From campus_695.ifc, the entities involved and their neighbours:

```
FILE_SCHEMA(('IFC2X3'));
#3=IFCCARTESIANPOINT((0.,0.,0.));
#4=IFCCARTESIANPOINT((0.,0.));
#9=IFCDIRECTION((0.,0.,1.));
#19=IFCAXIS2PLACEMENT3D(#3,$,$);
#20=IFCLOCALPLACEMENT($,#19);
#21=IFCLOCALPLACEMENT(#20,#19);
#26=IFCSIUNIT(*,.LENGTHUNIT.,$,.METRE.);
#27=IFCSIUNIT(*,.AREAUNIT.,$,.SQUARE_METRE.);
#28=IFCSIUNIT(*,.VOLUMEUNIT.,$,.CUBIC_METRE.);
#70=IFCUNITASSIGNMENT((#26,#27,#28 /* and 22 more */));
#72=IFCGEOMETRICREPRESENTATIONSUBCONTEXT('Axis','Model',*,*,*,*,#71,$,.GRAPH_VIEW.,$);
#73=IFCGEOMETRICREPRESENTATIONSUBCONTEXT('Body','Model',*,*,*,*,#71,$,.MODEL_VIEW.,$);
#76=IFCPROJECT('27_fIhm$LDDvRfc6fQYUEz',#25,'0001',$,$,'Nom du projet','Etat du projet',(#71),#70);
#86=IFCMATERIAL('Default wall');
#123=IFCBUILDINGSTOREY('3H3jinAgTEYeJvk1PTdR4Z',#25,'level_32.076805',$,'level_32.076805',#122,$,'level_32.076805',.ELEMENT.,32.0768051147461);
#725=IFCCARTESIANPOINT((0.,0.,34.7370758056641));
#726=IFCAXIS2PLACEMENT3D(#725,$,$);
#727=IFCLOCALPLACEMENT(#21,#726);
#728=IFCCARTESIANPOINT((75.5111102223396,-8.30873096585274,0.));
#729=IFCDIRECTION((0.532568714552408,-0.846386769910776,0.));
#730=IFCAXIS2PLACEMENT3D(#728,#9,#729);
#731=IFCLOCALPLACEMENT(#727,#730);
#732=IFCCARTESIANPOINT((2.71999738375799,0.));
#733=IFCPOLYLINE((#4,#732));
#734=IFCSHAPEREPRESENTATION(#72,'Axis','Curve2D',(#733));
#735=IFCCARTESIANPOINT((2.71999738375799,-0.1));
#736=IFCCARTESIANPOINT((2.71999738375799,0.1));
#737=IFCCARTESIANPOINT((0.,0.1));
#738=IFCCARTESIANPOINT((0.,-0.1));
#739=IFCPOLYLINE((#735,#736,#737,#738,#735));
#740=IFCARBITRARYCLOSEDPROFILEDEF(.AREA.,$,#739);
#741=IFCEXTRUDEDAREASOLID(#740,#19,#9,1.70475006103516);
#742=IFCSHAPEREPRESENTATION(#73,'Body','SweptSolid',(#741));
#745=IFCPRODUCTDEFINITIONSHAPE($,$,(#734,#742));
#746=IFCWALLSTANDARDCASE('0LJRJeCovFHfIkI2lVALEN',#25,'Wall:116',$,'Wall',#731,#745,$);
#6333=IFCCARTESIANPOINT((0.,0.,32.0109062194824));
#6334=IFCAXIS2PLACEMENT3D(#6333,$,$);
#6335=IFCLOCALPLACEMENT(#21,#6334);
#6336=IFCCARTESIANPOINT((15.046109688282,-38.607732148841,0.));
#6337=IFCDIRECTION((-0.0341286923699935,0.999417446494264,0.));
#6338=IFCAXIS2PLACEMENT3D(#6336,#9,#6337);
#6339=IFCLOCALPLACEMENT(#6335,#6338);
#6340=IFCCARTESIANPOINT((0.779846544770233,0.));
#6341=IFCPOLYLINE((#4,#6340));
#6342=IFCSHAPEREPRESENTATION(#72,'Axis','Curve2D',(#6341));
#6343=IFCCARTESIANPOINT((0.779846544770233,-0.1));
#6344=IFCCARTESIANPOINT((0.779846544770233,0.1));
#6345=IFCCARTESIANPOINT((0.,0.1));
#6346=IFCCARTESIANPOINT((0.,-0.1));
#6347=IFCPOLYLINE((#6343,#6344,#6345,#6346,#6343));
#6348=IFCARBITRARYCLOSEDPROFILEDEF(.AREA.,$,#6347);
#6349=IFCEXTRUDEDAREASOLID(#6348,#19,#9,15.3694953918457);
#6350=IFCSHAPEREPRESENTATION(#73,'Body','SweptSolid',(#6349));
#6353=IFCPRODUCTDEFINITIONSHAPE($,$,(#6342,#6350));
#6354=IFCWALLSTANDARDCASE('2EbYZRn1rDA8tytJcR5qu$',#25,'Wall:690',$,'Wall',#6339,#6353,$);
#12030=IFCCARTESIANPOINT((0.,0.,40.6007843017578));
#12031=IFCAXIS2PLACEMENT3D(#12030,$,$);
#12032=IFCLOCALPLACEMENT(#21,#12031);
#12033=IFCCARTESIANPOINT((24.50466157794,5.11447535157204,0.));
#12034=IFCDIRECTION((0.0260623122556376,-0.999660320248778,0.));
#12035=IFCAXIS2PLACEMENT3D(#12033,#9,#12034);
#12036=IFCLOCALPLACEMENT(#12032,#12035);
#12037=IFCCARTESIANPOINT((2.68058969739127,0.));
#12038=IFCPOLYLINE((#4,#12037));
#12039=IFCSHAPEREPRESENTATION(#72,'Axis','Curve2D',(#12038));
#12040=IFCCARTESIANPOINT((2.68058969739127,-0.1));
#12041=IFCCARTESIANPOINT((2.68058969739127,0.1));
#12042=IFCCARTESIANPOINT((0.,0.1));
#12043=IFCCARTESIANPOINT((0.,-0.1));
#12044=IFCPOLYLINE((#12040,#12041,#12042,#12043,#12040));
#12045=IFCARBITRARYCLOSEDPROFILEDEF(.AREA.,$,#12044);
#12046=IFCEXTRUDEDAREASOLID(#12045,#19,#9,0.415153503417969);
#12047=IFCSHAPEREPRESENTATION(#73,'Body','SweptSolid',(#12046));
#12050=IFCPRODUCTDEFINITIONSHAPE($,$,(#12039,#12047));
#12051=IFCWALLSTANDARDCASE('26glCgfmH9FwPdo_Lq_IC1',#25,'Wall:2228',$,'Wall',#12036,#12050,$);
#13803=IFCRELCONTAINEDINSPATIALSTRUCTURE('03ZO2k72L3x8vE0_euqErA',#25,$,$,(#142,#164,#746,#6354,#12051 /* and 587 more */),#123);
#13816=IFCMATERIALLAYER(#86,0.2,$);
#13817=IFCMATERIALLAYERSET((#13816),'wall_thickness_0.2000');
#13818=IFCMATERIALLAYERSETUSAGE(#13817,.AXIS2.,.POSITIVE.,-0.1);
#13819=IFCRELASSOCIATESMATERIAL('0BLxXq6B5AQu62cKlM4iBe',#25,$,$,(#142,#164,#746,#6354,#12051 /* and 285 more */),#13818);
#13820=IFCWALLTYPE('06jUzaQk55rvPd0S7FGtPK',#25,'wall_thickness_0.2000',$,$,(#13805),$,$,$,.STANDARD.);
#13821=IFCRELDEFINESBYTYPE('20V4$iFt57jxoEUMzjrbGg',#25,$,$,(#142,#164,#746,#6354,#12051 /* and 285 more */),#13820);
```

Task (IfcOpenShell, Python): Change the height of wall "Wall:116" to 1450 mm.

```python
import ifcopenshell
import ifcopenshell.geom
import ifcopenshell.util.representation
import ifcopenshell.util.shape

model = ifcopenshell.open("campus_695.ifc")
settings = ifcopenshell.geom.settings()


def volume(element):
    """Net volume in cubic metres, openings subtracted."""
    shape = ifcopenshell.geom.create_shape(settings, element)
    return ifcopenshell.util.shape.get_volume(shape.geometry)


wall = model.by_guid("0LJRJeCovFHfIkI2lVALEN")
before = volume(wall)

body = ifcopenshell.util.representation.get_representation(wall, "Model", "Body")
solid = body.Items[0]
old_height = solid.Depth
solid.Depth = 1.45
after = volume(wall)

print(f"height {old_height:g} -> {solid.Depth:g}, volume {before:.3f} -> {after:.3f} m3")

model.write("campus_695_edited.ifc")
```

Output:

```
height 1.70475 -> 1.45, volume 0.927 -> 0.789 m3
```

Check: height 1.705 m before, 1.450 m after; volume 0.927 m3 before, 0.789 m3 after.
